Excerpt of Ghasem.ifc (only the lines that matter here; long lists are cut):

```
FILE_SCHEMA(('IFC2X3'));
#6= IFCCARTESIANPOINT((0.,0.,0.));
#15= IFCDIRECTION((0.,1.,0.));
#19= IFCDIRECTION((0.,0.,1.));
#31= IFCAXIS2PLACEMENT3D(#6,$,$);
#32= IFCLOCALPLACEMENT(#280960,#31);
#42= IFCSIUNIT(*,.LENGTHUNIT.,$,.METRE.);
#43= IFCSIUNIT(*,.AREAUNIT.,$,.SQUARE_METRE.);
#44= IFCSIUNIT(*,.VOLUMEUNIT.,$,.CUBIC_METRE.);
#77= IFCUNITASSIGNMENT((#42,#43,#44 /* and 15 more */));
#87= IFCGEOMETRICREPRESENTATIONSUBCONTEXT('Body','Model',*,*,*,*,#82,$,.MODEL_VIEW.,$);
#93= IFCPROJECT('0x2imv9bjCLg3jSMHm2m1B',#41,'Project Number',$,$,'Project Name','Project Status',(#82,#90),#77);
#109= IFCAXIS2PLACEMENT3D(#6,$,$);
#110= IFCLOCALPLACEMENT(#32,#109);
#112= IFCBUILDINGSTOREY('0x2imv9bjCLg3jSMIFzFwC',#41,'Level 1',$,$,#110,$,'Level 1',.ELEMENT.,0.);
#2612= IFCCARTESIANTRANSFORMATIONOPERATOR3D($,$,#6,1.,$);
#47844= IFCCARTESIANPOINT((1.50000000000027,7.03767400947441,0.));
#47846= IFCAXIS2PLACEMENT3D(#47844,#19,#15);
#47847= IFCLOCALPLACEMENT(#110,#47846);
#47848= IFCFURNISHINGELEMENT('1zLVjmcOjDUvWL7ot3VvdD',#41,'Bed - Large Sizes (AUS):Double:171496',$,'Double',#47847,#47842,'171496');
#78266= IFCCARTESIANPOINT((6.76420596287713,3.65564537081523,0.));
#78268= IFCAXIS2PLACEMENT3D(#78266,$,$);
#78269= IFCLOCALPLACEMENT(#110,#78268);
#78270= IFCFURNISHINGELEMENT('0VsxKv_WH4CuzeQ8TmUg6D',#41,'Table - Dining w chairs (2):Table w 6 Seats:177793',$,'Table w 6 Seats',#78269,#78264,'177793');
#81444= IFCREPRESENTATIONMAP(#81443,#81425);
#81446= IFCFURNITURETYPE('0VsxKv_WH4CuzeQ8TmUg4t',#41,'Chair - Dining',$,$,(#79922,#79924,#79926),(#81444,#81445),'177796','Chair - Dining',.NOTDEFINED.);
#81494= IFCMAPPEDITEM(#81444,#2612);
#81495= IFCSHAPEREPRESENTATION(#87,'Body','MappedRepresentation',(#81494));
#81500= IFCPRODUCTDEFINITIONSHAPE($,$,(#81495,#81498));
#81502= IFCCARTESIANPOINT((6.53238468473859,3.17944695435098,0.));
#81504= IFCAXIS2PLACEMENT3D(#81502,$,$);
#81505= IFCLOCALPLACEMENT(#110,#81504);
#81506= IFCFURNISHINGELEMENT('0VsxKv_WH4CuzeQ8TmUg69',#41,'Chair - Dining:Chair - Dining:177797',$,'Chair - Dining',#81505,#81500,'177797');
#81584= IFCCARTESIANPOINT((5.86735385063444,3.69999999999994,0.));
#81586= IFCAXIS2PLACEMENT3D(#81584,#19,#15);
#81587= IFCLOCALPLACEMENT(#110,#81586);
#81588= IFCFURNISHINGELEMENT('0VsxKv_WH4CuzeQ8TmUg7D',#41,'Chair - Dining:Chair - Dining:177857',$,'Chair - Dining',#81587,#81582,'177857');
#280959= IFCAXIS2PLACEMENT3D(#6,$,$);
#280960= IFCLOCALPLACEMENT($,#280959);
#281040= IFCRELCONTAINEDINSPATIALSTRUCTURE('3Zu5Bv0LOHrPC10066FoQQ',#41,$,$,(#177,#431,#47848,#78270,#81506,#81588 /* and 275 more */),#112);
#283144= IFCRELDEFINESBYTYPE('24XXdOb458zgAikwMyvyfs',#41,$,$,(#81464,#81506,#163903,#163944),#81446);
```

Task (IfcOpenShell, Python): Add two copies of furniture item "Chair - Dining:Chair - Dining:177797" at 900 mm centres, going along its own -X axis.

```python
import ifcopenshell
import ifcopenshell.api.geometry
import ifcopenshell.api.root
import ifcopenshell.util.element
import ifcopenshell.util.placement
import ifcopenshell.util.unit

model = ifcopenshell.open("Ghasem.ifc")
unit_scale = ifcopenshell.util.unit.calculate_unit_scale(model)


def reuse_history(source, copy):
    """copy_class also copies each property set's owner history, people and application; keep the originals."""
    for rel in copy.IsDefinedBy:
        if rel.is_a("IfcRelDefinesByProperties") and (history := rel.RelatingPropertyDefinition.OwnerHistory):
            rel.RelatingPropertyDefinition.OwnerHistory = source.OwnerHistory
            ifcopenshell.util.element.remove_deep2(model, history)


source = model.by_id(81506)
base = ifcopenshell.util.placement.get_local_placement(source.ObjectPlacement)
step = -base[:3, 0] * 0.9 / unit_scale

for i in range(1, 3):
    copy = ifcopenshell.api.root.copy_class(model, product=source)
    copy.Representation = ifcopenshell.util.element.copy_deep(
        model, source.Representation, exclude=["IfcGeometricRepresentationContext", "IfcRepresentationMap"]
    )
    copy.Name = "Chair - Dining:Chair - Dining"
    copy.Tag = None
    reuse_history(source, copy)
    matrix = base.copy()
    matrix[:3, 3] += i * step
    print("added at", matrix[:3, 3].round(3) + 0.0)
    ifcopenshell.api.geometry.edit_object_placement(model, product=copy, matrix=matrix, is_si=False)

model.write("Ghasem_rev.ifc")
```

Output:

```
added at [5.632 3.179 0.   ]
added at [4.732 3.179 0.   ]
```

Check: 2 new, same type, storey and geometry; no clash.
